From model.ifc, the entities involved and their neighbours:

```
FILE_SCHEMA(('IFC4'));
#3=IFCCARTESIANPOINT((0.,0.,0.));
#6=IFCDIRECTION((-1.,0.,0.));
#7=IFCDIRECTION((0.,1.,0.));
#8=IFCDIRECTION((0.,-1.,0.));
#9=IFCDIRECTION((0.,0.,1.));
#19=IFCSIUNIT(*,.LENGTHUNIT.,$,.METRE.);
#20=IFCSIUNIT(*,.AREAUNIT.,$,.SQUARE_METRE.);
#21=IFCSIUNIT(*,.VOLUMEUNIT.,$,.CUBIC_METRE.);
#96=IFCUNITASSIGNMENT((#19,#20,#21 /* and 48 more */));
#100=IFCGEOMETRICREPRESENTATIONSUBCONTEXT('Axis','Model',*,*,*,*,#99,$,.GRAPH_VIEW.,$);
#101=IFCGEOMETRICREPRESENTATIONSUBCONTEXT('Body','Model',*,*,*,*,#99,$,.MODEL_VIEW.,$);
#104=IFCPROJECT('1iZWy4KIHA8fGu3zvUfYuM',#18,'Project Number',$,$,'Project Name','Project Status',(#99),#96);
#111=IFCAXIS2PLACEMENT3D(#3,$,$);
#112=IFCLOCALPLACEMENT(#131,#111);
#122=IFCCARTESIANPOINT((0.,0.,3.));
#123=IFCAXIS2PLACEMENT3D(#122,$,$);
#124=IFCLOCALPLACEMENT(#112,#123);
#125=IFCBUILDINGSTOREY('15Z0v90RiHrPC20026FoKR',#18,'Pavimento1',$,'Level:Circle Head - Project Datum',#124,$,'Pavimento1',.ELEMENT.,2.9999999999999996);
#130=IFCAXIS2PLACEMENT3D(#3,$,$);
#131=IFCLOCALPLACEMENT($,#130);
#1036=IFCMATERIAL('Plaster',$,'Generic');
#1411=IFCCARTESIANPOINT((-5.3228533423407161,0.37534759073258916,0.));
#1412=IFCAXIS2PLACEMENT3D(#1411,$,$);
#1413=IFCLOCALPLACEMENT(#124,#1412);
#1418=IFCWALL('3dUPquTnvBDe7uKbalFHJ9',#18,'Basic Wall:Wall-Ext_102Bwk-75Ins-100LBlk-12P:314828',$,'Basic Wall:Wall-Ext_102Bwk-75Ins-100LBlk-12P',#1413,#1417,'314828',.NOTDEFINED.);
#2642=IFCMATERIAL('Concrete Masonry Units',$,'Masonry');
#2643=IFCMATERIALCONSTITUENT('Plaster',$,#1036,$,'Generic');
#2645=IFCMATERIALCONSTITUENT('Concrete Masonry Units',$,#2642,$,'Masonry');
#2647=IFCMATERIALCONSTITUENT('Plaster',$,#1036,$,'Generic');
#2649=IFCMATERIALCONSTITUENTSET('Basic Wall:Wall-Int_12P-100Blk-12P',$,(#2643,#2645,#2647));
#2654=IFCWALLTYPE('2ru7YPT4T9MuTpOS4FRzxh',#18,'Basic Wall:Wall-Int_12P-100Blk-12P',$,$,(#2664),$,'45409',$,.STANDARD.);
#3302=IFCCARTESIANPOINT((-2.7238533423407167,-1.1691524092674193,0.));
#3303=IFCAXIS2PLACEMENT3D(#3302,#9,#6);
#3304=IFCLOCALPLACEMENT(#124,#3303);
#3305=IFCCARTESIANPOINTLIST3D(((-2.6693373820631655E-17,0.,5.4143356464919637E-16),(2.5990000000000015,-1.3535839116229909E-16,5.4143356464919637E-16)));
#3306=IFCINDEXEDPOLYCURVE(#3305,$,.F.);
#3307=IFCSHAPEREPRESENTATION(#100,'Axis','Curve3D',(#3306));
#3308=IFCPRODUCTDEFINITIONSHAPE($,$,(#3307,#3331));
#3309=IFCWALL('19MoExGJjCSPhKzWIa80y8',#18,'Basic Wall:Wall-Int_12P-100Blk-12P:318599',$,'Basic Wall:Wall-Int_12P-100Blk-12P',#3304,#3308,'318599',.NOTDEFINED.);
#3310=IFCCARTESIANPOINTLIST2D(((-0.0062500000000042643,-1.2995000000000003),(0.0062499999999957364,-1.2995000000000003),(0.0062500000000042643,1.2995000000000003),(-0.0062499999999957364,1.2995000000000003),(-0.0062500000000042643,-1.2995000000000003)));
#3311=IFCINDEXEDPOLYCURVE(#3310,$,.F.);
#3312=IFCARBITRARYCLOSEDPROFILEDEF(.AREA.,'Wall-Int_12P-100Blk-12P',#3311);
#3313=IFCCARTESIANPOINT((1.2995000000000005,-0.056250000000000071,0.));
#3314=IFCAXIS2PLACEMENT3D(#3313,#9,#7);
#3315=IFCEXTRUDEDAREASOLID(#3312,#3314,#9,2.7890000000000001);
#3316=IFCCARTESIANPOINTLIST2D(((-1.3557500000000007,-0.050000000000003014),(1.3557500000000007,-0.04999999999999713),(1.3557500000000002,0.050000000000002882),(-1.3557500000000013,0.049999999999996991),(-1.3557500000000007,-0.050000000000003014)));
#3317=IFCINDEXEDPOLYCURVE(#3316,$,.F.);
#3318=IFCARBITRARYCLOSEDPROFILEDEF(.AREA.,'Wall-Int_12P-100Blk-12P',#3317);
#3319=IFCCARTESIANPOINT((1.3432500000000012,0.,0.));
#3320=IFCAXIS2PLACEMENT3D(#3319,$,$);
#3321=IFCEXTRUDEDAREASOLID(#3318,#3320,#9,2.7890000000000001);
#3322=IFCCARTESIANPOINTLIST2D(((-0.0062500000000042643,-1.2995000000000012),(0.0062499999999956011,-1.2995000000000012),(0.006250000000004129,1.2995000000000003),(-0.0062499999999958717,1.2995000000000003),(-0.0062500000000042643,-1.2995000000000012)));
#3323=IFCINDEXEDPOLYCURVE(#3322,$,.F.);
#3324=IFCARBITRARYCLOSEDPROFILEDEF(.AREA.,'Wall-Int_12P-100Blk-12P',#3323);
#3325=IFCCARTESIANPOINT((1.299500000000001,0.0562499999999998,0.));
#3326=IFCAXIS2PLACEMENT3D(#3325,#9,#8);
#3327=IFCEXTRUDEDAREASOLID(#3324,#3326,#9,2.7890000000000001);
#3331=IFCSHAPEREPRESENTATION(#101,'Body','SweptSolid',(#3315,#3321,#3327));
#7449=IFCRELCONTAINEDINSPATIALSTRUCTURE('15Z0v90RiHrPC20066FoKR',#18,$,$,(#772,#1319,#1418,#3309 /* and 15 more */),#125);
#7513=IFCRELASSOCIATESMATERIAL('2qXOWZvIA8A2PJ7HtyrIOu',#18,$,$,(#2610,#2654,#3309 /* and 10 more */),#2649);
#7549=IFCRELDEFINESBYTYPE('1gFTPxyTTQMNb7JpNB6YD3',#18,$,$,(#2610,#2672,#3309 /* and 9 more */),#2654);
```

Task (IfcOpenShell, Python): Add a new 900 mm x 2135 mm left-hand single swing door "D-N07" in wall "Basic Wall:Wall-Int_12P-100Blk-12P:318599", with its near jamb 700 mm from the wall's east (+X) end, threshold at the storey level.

```python
import numpy as np
import ifcopenshell
import ifcopenshell.api.feature
import ifcopenshell.api.geometry
import ifcopenshell.api.root
import ifcopenshell.api.spatial
import ifcopenshell.geom
import ifcopenshell.util.element
import ifcopenshell.util.placement
import ifcopenshell.util.representation
import ifcopenshell.util.shape
import ifcopenshell.util.unit

model = ifcopenshell.open("model.ifc")
unit_scale = ifcopenshell.util.unit.calculate_unit_scale(model)
settings = ifcopenshell.geom.settings()


def volume(element):
    """Net volume in cubic metres, openings subtracted."""
    shape = ifcopenshell.geom.create_shape(settings, element)
    return ifcopenshell.util.shape.get_volume(shape.geometry)


wall = model.by_guid("19MoExGJjCSPhKzWIa80y8")
storey = ifcopenshell.util.element.get_container(wall, ifc_class="IfcBuildingStorey")
context = ifcopenshell.util.representation.get_context(model, "Model", "Body", "MODEL_VIEW")
before = volume(wall)

width, height, from_end, sill = 0.9, 2.135, 0.7, 0.0  # metres

# The wall runs along its own X axis, and the end named is its -X end.
wall_shape = ifcopenshell.geom.create_shape(settings, wall)
x, y, z = ifcopenshell.util.shape.get_vertices(wall_shape.geometry).T
start = x.min() + from_end
face, thickness = float(y.min()), float(y.max() - y.min())
wall_matrix = ifcopenshell.util.placement.get_local_placement(wall.ObjectPlacement)
level = ifcopenshell.util.placement.get_local_placement(storey.ObjectPlacement)[2, 3]


def in_wall(x, y):
    """Placement at x, y metres in the wall's axes, at sill height."""
    matrix = wall_matrix.copy()
    matrix[:, 3] = wall_matrix @ np.array([x / unit_scale, y / unit_scale, 0.0, 1.0])
    matrix[2, 3] = level + sill / unit_scale
    return matrix


# Opening: a box that overshoots both wall faces by 50 mm.
opening = ifcopenshell.api.root.create_entity(model, ifc_class="IfcOpeningElement", predefined_type="OPENING")
box = ifcopenshell.api.geometry.add_wall_representation(
    model, context=context, length=width, height=height, thickness=thickness + 0.1
)
ifcopenshell.api.geometry.assign_representation(model, product=opening, representation=box)
ifcopenshell.api.geometry.edit_object_placement(model, product=opening, matrix=in_wall(start, face - 0.05), is_si=False)
ifcopenshell.api.feature.add_feature(model, feature=opening, element=wall)

door = ifcopenshell.api.root.create_entity(model, ifc_class="IfcDoor", name="D-N07", predefined_type="DOOR")
door.OverallWidth, door.OverallHeight = width / unit_scale, height / unit_scale
door.OperationType = "SINGLE_SWING_LEFT"
body = ifcopenshell.api.geometry.add_door_representation(
    model,
    context=context,
    overall_width=door.OverallWidth,
    overall_height=door.OverallHeight,
    operation_type="SINGLE_SWING_LEFT",
    lining_properties={"LiningDepth": thickness / unit_scale, "ThresholdDepth": thickness / unit_scale},
)
ifcopenshell.api.geometry.assign_representation(model, product=door, representation=body)
ifcopenshell.api.spatial.assign_container(model, products=[door], relating_structure=storey)
ifcopenshell.api.feature.add_filling(model, opening=opening, element=door)

# The lining spans the wall, so the door starts at the wall face.
ifcopenshell.api.geometry.edit_object_placement(model, product=door, matrix=in_wall(start, face), is_si=False)

after = volume(wall)

print(f"wall volume {before:.3f} -> {after:.3f} m3")

model.write("model_v2.ifc")
```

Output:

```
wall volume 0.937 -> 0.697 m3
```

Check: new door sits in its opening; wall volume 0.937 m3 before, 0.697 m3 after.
